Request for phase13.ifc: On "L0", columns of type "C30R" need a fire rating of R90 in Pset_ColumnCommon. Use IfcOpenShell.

First a look at what the model holds.

```python
import ifcopenshell
import ifcopenshell.util.element

model = ifcopenshell.open("phase13.ifc")
print(model.schema)
storey = next(s for s in model.by_type("IfcBuildingStorey") if s.Name == "L0")
columns = [e for e in ifcopenshell.util.element.get_decomposition(storey) if e.is_a("IfcColumn")]
seen = {}
for e in columns:
    element_type = ifcopenshell.util.element.get_type(e)
    key = (element_type.Name if element_type != e and element_type else None, ifcopenshell.util.element.get_pset(e, "Pset_ColumnCommon", "FireRating"))
    seen[key] = seen.get(key, 0) + 1
for (name, value), count in sorted(seen.items(), key=str):
    print(count, "x", name, "|", value)
```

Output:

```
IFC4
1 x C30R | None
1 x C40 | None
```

```python
import ifcopenshell
import ifcopenshell.api.pset
import ifcopenshell.util.element

model = ifcopenshell.open("phase13.ifc")

storey = next(s for s in model.by_type("IfcBuildingStorey") if s.Name == "L0")
columns = [e for e in ifcopenshell.util.element.get_decomposition(storey) if e.is_a("IfcColumn")]

count = 0
for e in columns:
    element_type = ifcopenshell.util.element.get_type(e)
    if element_type in (None, e) or element_type.Name != "C30R":
        continue
    # add_pset returns the element's existing set when there is one.
    pset = ifcopenshell.api.pset.add_pset(model, product=e, name="Pset_ColumnCommon")
    ifcopenshell.api.pset.edit_pset(model, pset=pset, properties={"FireRating": "R90"})
    count += 1

print(count, "columns updated")

model.write("phase13-out.ifc")
```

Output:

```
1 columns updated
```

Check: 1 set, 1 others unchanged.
